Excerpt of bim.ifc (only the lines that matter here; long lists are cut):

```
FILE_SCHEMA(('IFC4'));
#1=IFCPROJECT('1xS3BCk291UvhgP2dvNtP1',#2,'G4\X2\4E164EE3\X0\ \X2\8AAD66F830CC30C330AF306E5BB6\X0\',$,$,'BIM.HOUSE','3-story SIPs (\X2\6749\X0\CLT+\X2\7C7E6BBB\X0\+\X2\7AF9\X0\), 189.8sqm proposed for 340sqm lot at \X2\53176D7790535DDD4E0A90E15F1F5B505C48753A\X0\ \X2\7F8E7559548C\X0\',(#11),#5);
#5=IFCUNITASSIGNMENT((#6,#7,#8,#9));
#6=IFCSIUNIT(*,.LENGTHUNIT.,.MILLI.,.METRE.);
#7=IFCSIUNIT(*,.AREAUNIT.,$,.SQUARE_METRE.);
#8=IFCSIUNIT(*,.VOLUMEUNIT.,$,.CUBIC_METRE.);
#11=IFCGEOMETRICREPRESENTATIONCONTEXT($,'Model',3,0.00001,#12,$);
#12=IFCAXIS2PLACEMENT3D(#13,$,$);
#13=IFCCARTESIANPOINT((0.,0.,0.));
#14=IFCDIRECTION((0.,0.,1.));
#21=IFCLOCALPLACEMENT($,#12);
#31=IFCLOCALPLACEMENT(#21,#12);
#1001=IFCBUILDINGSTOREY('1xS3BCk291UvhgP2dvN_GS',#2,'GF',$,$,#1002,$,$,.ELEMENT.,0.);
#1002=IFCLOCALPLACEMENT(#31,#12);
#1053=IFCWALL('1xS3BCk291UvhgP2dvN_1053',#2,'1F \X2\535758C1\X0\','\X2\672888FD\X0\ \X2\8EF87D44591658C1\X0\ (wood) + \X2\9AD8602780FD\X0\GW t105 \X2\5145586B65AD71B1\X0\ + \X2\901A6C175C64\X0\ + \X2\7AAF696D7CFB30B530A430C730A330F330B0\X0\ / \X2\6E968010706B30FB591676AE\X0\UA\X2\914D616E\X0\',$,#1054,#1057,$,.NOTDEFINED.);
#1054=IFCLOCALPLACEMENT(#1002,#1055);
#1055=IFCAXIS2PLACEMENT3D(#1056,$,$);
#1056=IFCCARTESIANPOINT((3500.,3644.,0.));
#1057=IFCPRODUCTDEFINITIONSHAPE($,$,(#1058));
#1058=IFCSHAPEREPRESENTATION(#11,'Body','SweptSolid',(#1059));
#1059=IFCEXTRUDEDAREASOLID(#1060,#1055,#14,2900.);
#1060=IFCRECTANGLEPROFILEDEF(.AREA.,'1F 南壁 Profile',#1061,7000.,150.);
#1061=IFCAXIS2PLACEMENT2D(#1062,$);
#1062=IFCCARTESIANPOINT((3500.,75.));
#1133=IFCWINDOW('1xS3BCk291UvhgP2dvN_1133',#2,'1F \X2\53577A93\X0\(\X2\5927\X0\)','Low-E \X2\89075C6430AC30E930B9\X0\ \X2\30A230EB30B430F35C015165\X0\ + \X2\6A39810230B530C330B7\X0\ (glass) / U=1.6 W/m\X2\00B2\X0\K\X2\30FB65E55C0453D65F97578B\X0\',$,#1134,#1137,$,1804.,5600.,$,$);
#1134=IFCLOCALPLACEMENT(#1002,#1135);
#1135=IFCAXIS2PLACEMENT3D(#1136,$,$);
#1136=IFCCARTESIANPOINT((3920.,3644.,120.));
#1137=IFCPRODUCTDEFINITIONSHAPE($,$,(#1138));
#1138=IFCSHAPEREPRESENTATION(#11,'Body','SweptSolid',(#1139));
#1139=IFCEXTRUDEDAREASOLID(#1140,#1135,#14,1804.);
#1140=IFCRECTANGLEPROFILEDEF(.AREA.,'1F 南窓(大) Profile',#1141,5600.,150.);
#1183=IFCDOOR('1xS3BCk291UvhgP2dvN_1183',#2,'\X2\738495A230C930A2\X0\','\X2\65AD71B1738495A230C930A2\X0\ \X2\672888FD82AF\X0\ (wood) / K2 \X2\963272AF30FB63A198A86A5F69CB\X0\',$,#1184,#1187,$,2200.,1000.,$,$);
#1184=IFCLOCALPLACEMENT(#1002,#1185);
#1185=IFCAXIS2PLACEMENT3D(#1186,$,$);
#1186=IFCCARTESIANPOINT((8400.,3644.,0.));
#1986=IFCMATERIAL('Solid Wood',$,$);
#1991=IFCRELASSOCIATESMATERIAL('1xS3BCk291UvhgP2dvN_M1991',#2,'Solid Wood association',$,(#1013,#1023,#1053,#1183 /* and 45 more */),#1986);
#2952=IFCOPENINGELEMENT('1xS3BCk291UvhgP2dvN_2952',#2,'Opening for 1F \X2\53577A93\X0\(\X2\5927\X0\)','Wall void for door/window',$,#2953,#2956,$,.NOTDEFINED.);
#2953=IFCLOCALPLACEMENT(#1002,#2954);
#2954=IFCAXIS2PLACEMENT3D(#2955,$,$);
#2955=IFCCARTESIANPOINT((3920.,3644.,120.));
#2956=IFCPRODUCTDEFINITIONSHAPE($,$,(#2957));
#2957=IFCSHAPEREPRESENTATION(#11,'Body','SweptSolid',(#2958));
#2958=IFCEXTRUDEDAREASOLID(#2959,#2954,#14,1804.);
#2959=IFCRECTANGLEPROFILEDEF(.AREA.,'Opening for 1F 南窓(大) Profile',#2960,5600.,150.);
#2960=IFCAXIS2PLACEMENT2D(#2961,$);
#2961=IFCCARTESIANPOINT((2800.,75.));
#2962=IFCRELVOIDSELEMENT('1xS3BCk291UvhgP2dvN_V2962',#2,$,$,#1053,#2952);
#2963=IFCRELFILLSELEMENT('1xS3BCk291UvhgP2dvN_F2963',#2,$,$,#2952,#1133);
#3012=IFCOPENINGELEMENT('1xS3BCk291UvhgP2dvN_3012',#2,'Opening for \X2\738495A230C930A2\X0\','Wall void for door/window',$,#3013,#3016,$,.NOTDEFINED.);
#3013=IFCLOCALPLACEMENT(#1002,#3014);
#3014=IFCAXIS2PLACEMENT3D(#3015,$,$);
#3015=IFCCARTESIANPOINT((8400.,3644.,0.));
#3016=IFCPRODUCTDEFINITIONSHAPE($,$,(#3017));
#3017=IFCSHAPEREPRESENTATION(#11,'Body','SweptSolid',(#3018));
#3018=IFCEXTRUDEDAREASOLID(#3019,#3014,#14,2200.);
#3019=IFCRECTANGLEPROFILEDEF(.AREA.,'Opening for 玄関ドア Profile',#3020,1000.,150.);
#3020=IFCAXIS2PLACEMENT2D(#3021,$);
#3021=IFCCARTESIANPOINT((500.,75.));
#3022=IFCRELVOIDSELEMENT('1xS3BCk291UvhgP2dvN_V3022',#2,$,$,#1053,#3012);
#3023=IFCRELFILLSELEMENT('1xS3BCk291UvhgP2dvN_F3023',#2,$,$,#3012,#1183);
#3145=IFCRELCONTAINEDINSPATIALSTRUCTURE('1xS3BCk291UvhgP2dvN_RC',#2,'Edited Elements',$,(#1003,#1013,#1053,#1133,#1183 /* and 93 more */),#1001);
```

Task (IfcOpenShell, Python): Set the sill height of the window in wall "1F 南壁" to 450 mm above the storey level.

```python
import numpy as np
import ifcopenshell
import ifcopenshell.api.geometry
import ifcopenshell.geom
import ifcopenshell.util.element
import ifcopenshell.util.placement
import ifcopenshell.util.shape
import ifcopenshell.util.unit

model = ifcopenshell.open("bim.ifc")
unit_scale = ifcopenshell.util.unit.calculate_unit_scale(model)

window = model.by_id(1133)
opening = window.FillsVoids[0].RelatingOpeningElement
storey = ifcopenshell.util.element.get_container(window, ifc_class="IfcBuildingStorey")
level = ifcopenshell.util.placement.get_local_placement(storey.ObjectPlacement)[2, 3]

# The opening's origin need not be at the sill, so measure its lowest point.
shape = ifcopenshell.geom.create_shape(ifcopenshell.geom.settings(), opening)
bottom = ifcopenshell.util.shape.get_shape_bottom_elevation(shape, shape.geometry) / unit_scale
dz = level + 0.45 / unit_scale - bottom

shift = np.array([0.0, 0.0, dz])
# The window is not placed relative to its opening, so move both.
for product in (opening, window):
    matrix = ifcopenshell.util.placement.get_local_placement(product.ObjectPlacement)
    matrix[:3, 3] += shift
    ifcopenshell.api.geometry.edit_object_placement(model, product=product, matrix=matrix, is_si=False)

print(f"moved by {dz * unit_scale:+.3f} m")

model.write("bim_edited.ifc")
```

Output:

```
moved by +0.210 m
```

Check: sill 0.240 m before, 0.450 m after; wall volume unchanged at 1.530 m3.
